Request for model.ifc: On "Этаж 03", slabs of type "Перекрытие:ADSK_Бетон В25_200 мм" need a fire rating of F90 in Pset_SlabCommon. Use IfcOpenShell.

First a look at what the model holds.

```python
import ifcopenshell
import ifcopenshell.util.element

model = ifcopenshell.open("model.ifc")
print(model.schema)
storey = next(s for s in model.by_type("IfcBuildingStorey") if s.Name == "Этаж 03")
slabs = [e for e in ifcopenshell.util.element.get_decomposition(storey) if e.is_a("IfcSlab")]
seen = {}
for e in slabs:
    element_type = ifcopenshell.util.element.get_type(e)
    key = (element_type.Name if element_type != e and element_type else None, ifcopenshell.util.element.get_pset(e, "Pset_SlabCommon", "FireRating"))
    seen[key] = seen.get(key, 0) + 1
for (name, value), count in sorted(seen.items(), key=str):
    print(count, "x", name, "|", value)
```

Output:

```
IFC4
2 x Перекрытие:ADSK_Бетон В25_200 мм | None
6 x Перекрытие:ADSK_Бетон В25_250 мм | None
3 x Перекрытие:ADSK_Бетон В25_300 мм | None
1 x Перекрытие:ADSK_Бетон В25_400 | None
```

```python
import ifcopenshell
import ifcopenshell.api.pset
import ifcopenshell.util.element

model = ifcopenshell.open("model.ifc")

storey = next(s for s in model.by_type("IfcBuildingStorey") if s.Name == "Этаж 03")
slabs = [e for e in ifcopenshell.util.element.get_decomposition(storey) if e.is_a("IfcSlab")]

count = 0
for e in slabs:
    element_type = ifcopenshell.util.element.get_type(e)
    if element_type in (None, e) or element_type.Name != "Перекрытие:ADSK_Бетон В25_200 мм":
        continue
    # add_pset returns the element's existing set when there is one.
    pset = ifcopenshell.api.pset.add_pset(model, product=e, name="Pset_SlabCommon")
    ifcopenshell.api.pset.edit_pset(model, pset=pset, properties={"FireRating": "F90"})
    count += 1

print(count, "slabs updated")

model.write("model-out.ifc")
```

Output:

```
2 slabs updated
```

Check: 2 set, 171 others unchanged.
